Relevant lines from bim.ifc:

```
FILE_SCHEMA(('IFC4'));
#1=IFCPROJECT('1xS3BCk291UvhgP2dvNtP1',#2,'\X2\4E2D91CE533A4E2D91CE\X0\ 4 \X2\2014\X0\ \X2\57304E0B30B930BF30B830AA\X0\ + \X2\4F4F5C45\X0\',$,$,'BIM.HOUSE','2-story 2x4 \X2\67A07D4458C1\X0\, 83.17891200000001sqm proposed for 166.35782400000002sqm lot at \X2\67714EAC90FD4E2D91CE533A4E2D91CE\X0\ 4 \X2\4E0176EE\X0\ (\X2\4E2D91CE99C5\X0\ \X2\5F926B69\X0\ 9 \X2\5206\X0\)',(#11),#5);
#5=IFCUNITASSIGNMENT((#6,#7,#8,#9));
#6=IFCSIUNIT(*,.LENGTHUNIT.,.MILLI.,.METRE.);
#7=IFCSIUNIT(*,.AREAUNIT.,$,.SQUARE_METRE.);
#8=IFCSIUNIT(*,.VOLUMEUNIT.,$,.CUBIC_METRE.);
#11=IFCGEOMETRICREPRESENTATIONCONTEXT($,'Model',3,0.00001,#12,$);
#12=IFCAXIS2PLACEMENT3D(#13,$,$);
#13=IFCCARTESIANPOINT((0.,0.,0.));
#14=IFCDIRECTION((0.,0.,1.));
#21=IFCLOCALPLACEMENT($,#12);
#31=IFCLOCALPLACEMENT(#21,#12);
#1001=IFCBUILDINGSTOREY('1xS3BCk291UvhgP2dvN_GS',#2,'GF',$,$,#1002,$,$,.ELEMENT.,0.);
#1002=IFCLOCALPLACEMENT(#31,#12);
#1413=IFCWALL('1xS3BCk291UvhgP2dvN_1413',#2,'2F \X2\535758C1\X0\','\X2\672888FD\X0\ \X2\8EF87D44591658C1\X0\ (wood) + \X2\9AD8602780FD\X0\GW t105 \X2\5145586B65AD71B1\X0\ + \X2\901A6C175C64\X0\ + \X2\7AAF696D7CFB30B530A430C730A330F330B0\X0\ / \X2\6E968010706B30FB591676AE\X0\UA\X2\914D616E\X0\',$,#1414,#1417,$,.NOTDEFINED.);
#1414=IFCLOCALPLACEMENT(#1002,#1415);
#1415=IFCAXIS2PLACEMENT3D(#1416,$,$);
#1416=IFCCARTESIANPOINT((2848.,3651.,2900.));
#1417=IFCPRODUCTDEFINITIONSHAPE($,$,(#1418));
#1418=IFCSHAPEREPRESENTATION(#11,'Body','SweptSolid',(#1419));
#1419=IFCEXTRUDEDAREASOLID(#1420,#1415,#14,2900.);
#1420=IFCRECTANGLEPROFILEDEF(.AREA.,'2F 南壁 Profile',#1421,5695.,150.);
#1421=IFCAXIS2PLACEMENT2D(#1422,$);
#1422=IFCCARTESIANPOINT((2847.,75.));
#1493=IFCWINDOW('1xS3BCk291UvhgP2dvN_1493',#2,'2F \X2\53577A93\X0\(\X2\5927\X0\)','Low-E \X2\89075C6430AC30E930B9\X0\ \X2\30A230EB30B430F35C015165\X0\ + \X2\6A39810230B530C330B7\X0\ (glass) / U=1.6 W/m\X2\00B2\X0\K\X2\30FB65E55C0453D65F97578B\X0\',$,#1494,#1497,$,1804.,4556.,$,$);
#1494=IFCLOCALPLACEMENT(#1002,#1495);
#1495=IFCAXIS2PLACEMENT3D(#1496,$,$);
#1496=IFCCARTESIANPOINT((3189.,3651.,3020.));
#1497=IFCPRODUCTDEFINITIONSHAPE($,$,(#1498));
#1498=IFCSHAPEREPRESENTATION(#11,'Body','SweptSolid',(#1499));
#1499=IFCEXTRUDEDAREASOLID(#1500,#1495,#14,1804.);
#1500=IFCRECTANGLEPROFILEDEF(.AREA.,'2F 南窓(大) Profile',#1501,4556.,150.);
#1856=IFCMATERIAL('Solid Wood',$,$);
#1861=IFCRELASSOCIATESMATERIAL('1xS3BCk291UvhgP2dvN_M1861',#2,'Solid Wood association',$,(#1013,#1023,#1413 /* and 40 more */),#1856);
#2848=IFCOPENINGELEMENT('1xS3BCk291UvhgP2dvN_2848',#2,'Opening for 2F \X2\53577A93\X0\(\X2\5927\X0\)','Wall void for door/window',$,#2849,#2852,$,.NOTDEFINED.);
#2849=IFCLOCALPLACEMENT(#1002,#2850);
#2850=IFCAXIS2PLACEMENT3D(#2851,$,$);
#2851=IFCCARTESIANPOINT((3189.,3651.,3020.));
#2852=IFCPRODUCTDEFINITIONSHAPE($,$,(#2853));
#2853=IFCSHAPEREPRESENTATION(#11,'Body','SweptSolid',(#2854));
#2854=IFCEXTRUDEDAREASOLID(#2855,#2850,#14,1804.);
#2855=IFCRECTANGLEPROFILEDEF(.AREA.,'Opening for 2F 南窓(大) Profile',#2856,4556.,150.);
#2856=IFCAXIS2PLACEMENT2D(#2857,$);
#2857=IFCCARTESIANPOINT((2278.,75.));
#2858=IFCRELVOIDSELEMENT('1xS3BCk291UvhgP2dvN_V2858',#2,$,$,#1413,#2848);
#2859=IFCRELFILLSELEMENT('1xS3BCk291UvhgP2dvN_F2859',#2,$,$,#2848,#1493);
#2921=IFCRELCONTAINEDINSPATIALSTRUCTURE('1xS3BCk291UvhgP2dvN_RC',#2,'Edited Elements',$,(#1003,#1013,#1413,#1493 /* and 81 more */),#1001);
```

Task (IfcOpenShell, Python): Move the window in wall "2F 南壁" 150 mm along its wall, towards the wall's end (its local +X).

```python
import ifcopenshell
import ifcopenshell.api.geometry
import ifcopenshell.util.placement
import ifcopenshell.util.unit

model = ifcopenshell.open("bim.ifc")
unit_scale = ifcopenshell.util.unit.calculate_unit_scale(model)

window = model.by_id(1493)
opening = window.FillsVoids[0].RelatingOpeningElement
wall = opening.VoidsElements[0].RelatingBuildingElement

wall_matrix = ifcopenshell.util.placement.get_local_placement(wall.ObjectPlacement)
shift = wall_matrix[:3, 0] * 0.15 / unit_scale
before = ifcopenshell.util.placement.get_local_placement(window.ObjectPlacement)[:3, 3].copy()

# The window is not placed relative to its opening, so move both.
for product in (opening, window):
    matrix = ifcopenshell.util.placement.get_local_placement(product.ObjectPlacement)
    matrix[:3, 3] += shift
    ifcopenshell.api.geometry.edit_object_placement(model, product=product, matrix=matrix, is_si=False)

after = ifcopenshell.util.placement.get_local_placement(window.ObjectPlacement)[:3, 3]
print("window moved by", (after - before).round(3) + 0.0)

model.write("bim_v2.ifc")
```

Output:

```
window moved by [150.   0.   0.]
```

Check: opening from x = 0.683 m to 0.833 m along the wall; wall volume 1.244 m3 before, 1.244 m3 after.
